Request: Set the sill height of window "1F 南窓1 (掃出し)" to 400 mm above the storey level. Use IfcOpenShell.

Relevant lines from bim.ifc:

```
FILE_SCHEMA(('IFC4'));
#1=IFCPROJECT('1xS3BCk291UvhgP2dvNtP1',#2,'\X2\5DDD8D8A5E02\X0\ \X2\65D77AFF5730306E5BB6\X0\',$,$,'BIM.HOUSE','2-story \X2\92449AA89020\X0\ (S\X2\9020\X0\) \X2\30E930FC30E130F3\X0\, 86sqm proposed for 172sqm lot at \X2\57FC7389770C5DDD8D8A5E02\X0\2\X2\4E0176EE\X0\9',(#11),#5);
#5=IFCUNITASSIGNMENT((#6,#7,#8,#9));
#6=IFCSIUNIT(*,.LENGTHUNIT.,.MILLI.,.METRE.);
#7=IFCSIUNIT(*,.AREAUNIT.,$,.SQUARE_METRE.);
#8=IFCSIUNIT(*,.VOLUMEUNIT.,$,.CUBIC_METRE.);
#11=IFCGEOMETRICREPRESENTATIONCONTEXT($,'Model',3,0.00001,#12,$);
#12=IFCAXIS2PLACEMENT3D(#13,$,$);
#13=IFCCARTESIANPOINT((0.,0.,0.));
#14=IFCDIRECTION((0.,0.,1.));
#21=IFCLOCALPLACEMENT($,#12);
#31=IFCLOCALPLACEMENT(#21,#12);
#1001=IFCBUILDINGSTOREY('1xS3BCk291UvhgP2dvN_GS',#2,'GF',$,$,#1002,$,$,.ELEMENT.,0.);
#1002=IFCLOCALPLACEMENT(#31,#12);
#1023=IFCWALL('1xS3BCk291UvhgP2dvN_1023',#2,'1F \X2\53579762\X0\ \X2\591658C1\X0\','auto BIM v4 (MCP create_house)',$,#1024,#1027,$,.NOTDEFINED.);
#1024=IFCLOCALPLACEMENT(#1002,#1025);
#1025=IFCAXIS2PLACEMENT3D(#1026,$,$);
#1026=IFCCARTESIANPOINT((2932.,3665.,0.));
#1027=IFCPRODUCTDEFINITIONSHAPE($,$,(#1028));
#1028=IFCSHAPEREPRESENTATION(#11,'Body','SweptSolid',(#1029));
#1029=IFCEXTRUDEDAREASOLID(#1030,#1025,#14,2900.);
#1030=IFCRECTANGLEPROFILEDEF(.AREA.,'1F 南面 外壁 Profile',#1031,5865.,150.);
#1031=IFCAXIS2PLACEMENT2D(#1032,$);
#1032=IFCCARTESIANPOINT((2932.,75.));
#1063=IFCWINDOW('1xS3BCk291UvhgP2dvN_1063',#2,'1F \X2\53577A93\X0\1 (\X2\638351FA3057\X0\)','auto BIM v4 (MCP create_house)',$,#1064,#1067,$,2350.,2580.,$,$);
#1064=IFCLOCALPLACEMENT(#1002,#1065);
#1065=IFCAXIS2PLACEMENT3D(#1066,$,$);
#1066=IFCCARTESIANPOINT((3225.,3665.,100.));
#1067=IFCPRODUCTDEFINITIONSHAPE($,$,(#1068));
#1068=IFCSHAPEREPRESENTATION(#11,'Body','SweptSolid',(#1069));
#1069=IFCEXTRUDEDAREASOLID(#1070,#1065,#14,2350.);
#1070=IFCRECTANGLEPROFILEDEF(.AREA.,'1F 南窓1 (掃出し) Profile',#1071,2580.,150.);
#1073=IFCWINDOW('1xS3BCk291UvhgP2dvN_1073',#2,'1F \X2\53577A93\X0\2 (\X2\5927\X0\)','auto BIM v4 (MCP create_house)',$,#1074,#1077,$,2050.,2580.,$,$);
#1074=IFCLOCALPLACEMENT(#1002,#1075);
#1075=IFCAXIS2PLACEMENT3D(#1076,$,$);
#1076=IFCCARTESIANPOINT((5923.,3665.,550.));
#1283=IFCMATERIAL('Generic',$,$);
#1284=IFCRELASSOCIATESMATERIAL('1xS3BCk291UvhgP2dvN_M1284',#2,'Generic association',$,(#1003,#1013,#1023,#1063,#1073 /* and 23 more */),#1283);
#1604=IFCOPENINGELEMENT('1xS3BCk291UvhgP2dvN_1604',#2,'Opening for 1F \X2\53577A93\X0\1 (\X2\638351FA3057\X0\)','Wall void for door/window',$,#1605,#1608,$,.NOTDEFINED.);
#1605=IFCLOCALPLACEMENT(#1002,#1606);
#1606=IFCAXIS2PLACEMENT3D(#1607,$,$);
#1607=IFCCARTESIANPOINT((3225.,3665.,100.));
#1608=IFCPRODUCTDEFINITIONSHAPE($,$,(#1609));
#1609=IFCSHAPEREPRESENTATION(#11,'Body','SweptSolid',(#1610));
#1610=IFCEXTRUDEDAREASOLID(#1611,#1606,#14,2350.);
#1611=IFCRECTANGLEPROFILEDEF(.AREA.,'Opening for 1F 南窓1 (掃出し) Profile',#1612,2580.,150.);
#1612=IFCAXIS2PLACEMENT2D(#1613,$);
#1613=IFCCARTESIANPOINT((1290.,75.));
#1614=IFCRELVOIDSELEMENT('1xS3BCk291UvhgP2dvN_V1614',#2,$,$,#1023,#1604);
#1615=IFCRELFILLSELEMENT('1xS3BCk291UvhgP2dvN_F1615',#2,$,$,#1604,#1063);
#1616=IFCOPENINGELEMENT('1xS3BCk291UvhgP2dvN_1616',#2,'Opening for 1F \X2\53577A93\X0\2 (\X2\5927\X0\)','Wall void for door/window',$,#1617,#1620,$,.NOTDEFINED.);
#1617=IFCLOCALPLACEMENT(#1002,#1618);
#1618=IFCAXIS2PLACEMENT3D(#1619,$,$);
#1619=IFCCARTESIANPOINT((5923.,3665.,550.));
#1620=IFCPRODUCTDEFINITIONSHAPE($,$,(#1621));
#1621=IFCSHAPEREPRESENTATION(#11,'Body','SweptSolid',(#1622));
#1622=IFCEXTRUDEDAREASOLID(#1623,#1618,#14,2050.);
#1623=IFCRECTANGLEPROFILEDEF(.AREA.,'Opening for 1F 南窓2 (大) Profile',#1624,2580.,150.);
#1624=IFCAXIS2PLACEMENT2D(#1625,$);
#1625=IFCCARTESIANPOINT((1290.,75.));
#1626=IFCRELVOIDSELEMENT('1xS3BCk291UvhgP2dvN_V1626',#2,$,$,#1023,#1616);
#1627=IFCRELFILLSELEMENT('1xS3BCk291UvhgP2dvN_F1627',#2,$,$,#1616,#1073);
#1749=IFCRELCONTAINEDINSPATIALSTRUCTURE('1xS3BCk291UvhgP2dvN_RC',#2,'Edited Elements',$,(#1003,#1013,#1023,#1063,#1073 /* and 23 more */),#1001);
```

```python
import numpy as np
import ifcopenshell
import ifcopenshell.api.geometry
import ifcopenshell.geom
import ifcopenshell.util.element
import ifcopenshell.util.placement
import ifcopenshell.util.shape
import ifcopenshell.util.unit

model = ifcopenshell.open("bim.ifc")
unit_scale = ifcopenshell.util.unit.calculate_unit_scale(model)

window = model.by_guid("1xS3BCk291UvhgP2dvN_1063")
opening = window.FillsVoids[0].RelatingOpeningElement
storey = ifcopenshell.util.element.get_container(window, ifc_class="IfcBuildingStorey")
level = ifcopenshell.util.placement.get_local_placement(storey.ObjectPlacement)[2, 3]

# The opening's origin need not be at the sill, so measure its lowest point.
shape = ifcopenshell.geom.create_shape(ifcopenshell.geom.settings(), opening)
bottom = ifcopenshell.util.shape.get_shape_bottom_elevation(shape, shape.geometry) / unit_scale
dz = level + 400.0 - bottom

shift = np.array([0.0, 0.0, dz])
# The window is not placed relative to its opening, so move both.
for product in (opening, window):
    matrix = ifcopenshell.util.placement.get_local_placement(product.ObjectPlacement)
    matrix[:3, 3] += shift
    ifcopenshell.api.geometry.edit_object_placement(model, product=product, matrix=matrix, is_si=False)

print(f"moved by {dz * unit_scale:+.3f} m")

model.write("bim_updated.ifc")
```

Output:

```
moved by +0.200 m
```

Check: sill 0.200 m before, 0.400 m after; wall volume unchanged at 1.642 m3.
